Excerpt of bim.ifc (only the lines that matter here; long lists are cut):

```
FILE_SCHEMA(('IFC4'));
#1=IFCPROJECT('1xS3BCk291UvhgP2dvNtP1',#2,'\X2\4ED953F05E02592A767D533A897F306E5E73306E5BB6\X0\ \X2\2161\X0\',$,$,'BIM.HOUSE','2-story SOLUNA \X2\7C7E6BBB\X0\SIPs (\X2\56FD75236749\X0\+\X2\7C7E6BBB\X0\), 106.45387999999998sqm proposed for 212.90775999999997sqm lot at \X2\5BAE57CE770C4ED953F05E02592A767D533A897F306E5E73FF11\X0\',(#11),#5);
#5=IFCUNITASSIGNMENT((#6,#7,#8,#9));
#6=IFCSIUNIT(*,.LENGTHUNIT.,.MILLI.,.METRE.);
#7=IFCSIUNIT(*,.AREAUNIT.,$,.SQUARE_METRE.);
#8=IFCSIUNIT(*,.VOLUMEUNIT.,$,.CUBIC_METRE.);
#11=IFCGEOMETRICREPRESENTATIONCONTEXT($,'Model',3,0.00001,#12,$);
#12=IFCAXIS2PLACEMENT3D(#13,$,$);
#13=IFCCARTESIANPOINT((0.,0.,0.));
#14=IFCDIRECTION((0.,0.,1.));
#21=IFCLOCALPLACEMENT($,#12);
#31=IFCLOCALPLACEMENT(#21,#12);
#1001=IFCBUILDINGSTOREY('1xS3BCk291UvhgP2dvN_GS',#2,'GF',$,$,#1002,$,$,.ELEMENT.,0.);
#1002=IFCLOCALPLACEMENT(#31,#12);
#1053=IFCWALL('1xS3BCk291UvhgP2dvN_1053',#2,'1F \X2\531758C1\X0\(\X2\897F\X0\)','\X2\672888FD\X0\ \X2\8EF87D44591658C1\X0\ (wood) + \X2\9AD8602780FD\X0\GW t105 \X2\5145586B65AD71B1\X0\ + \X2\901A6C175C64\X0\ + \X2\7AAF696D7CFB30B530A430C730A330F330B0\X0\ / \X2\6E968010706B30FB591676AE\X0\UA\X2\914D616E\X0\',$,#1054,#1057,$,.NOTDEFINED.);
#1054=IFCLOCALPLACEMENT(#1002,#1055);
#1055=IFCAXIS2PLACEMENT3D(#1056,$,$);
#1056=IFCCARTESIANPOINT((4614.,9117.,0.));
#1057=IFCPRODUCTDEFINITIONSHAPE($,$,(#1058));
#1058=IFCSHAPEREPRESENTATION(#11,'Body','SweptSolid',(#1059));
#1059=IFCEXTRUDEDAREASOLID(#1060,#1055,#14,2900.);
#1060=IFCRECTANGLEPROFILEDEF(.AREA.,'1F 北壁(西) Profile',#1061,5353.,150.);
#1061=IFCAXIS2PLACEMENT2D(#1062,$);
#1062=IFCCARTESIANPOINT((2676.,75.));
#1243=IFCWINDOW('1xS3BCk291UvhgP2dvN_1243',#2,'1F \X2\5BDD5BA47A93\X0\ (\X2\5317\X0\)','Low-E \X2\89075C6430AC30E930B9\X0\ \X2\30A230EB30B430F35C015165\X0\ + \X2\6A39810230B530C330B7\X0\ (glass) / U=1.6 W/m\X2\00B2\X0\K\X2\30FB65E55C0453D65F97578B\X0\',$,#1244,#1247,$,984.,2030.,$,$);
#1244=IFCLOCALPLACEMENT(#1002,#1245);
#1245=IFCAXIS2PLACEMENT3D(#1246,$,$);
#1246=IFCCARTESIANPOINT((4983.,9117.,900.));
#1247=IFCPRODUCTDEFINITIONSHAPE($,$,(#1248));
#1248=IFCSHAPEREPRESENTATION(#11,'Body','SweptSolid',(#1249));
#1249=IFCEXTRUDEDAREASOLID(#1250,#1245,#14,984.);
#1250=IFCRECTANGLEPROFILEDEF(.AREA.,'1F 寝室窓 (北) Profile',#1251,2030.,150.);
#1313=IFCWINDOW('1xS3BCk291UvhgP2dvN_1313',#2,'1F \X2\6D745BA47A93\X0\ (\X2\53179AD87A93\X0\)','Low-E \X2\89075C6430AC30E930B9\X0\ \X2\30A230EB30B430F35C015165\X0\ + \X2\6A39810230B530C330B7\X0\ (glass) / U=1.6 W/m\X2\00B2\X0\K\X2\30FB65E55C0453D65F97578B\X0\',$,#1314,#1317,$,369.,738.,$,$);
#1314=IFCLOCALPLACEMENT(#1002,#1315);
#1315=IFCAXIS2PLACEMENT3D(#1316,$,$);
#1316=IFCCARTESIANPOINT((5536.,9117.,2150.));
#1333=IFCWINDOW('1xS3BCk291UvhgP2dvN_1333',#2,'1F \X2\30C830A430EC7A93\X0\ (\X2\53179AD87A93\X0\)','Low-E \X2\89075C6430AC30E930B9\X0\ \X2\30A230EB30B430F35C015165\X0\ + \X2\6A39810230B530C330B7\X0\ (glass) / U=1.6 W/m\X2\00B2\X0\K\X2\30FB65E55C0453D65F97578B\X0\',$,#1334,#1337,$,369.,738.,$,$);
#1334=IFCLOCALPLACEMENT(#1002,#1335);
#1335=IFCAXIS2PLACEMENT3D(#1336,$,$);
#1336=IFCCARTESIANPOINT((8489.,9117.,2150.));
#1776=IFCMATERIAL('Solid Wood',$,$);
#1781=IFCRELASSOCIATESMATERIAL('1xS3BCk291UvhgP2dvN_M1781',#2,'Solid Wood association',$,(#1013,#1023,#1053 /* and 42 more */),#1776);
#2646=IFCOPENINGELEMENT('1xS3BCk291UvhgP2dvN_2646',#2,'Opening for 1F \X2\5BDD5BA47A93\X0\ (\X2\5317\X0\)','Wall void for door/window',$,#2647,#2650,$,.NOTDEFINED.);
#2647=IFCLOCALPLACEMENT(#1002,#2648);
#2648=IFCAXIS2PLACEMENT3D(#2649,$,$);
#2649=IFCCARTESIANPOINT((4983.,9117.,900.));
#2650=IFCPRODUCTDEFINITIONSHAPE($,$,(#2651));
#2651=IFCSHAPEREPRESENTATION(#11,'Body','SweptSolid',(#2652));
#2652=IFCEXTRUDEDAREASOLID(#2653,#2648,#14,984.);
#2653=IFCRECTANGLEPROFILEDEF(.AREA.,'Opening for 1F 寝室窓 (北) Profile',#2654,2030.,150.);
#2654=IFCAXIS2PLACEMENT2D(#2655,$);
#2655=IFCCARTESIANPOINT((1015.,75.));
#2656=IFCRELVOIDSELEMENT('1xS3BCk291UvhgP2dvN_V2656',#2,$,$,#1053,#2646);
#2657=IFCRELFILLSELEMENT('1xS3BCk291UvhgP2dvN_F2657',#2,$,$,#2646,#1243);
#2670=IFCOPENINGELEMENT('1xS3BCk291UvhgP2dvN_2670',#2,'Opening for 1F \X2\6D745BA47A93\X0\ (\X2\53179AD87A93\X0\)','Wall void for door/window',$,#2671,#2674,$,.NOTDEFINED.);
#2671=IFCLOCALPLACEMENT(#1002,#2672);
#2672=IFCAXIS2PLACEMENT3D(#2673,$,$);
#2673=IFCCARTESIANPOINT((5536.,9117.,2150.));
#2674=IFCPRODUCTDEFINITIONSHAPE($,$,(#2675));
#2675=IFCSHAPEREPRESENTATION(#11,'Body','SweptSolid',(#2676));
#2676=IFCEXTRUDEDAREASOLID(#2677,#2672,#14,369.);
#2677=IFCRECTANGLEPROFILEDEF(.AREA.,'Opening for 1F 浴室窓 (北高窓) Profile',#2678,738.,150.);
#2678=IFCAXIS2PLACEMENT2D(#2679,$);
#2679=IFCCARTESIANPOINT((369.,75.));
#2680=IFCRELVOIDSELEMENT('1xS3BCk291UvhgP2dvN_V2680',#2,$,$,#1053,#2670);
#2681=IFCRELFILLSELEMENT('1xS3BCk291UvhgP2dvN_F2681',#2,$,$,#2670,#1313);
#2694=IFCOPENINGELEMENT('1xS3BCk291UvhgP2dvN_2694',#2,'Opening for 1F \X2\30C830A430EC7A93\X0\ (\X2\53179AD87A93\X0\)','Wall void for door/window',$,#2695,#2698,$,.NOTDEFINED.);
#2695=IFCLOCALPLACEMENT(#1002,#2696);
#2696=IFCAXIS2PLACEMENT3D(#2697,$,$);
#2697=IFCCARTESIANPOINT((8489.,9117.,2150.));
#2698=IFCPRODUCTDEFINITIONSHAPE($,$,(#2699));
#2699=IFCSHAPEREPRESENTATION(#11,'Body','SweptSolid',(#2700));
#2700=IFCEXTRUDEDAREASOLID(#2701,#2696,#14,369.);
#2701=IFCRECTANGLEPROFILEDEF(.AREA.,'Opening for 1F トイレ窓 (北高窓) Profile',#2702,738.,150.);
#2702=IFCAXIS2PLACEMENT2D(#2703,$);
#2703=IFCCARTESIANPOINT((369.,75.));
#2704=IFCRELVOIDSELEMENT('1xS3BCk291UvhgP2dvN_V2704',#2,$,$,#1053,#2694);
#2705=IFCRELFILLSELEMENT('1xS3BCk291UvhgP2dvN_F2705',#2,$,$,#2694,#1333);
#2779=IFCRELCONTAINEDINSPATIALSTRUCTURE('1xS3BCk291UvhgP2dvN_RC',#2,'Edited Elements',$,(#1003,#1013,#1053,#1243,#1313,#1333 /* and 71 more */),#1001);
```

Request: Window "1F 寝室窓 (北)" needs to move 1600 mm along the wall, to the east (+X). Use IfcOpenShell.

```python
import ifcopenshell
import ifcopenshell.api.geometry
import ifcopenshell.util.placement
import ifcopenshell.util.unit

model = ifcopenshell.open("bim.ifc")
unit_scale = ifcopenshell.util.unit.calculate_unit_scale(model)

window = model.by_guid("1xS3BCk291UvhgP2dvN_1243")
opening = window.FillsVoids[0].RelatingOpeningElement
wall = opening.VoidsElements[0].RelatingBuildingElement

wall_matrix = ifcopenshell.util.placement.get_local_placement(wall.ObjectPlacement)
shift = wall_matrix[:3, 0] * 1.6 / unit_scale
before = ifcopenshell.util.placement.get_local_placement(window.ObjectPlacement)[:3, 3].copy()

# The window is not placed relative to its opening, so move both.
for product in (opening, window):
    matrix = ifcopenshell.util.placement.get_local_placement(product.ObjectPlacement)
    matrix[:3, 3] += shift
    ifcopenshell.api.geometry.edit_object_placement(model, product=product, matrix=matrix, is_si=False)

after = ifcopenshell.util.placement.get_local_placement(window.ObjectPlacement)[:3, 3]
print("window moved by", (after - before).round(3) + 0.0)

model.write("bim_rev.ifc")
```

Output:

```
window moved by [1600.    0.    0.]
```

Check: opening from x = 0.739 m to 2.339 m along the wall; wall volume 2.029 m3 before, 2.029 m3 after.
